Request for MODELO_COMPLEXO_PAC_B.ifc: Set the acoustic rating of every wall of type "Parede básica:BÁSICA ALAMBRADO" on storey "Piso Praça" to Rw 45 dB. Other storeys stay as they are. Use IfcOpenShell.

First a look at what the model holds.

```python
import ifcopenshell
import ifcopenshell.util.element

model = ifcopenshell.open("MODELO_COMPLEXO_PAC_B.ifc")
print(model.schema)
storey = next(s for s in model.by_type("IfcBuildingStorey") if s.Name == "Piso Praça")
walls = [e for e in ifcopenshell.util.element.get_decomposition(storey) if e.is_a("IfcWall")]
seen = {}
for e in walls:
    element_type = ifcopenshell.util.element.get_type(e)
    key = (element_type.Name if element_type != e and element_type else None, ifcopenshell.util.element.get_pset(e, "Pset_WallCommon", "AcousticRating"))
    seen[key] = seen.get(key, 0) + 1
for (name, value), count in sorted(seen.items(), key=str):
    print(count, "x", name, "|", value)
```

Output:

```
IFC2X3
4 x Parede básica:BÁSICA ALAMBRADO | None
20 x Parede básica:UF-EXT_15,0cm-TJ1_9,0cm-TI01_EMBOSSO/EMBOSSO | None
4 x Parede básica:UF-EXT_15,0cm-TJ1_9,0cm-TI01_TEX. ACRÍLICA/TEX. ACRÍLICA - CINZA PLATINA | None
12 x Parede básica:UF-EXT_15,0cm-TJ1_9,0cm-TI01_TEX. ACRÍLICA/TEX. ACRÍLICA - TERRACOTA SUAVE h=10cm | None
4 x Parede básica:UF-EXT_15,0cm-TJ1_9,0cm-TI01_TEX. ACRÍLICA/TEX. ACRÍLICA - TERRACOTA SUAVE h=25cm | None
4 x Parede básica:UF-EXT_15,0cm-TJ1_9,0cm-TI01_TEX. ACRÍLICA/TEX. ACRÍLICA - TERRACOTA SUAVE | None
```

```python
import ifcopenshell
import ifcopenshell.api.pset
import ifcopenshell.util.element

model = ifcopenshell.open("MODELO_COMPLEXO_PAC_B.ifc")

storey = next(s for s in model.by_type("IfcBuildingStorey") if s.Name == "Piso Praça")
walls = [e for e in ifcopenshell.util.element.get_decomposition(storey) if e.is_a("IfcWall")]

count = 0
for e in walls:
    element_type = ifcopenshell.util.element.get_type(e)
    if element_type in (None, e) or element_type.Name != "Parede básica:BÁSICA ALAMBRADO":
        continue
    # add_pset returns the element's existing set when there is one.
    pset = ifcopenshell.api.pset.add_pset(model, product=e, name="Pset_WallCommon")
    ifcopenshell.api.pset.edit_pset(model, pset=pset, properties={"AcousticRating": "Rw 45 dB"})
    count += 1

print(count, "walls updated")

model.write("MODELO_COMPLEXO_PAC_B_v2.ifc")
```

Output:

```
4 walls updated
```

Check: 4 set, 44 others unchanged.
